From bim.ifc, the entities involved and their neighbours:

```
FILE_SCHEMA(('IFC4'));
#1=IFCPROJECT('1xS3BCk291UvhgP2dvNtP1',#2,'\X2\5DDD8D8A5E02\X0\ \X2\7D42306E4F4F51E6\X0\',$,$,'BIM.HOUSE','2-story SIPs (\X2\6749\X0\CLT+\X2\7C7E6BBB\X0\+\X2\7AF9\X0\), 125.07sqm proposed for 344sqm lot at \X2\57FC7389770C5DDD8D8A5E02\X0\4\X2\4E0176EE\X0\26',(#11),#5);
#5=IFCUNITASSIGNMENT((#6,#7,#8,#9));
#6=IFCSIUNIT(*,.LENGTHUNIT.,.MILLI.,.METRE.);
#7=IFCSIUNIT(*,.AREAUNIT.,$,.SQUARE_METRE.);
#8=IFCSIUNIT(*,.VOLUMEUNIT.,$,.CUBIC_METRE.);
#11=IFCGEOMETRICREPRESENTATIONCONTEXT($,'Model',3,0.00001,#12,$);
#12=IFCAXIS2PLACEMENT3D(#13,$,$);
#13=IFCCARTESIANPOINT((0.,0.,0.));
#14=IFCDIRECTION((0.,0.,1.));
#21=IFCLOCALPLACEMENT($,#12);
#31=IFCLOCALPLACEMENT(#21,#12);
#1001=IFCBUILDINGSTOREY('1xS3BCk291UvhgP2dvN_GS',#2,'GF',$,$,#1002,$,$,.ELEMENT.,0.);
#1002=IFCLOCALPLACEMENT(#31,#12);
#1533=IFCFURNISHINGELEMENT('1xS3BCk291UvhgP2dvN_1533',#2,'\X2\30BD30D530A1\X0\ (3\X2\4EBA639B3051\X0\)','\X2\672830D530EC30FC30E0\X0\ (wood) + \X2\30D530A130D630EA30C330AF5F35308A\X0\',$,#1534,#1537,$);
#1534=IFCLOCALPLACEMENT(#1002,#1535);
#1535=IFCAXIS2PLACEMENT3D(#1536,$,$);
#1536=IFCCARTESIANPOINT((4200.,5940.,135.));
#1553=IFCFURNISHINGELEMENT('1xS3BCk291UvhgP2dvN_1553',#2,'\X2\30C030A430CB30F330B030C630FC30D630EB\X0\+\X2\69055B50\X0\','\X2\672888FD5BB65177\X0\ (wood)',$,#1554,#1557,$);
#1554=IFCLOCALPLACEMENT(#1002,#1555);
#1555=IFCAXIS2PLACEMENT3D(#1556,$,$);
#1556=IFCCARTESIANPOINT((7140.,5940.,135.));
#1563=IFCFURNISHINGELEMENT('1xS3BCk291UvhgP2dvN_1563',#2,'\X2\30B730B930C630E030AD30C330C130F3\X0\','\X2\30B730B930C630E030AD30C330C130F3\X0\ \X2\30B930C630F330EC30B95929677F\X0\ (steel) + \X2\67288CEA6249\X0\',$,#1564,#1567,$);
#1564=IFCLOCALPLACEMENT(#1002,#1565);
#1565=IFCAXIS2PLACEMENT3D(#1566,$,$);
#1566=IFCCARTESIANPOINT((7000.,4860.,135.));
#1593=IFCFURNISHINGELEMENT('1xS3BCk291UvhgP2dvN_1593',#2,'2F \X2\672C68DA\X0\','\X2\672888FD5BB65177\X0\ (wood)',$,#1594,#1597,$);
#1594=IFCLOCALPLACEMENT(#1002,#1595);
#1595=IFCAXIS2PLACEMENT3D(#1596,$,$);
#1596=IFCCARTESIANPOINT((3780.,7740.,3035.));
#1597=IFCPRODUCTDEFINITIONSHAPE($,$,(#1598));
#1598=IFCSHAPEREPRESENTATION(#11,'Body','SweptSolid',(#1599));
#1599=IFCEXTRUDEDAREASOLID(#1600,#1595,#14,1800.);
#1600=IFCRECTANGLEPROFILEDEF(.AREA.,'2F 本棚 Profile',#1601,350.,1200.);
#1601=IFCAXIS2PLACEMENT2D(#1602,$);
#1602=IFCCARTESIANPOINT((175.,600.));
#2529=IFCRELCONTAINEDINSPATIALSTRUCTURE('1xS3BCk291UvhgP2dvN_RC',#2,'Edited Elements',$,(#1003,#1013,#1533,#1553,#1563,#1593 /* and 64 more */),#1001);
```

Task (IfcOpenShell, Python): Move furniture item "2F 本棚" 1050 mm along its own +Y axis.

```python
import ifcopenshell
import ifcopenshell.api.geometry
import ifcopenshell.util.placement
import ifcopenshell.util.unit

model = ifcopenshell.open("bim.ifc")
unit_scale = ifcopenshell.util.unit.calculate_unit_scale(model)

item = model.by_id(1593)
matrix = ifcopenshell.util.placement.get_local_placement(item.ObjectPlacement)
matrix[:3, 3] += matrix[:3, 1] * 1.05 / unit_scale
ifcopenshell.api.geometry.edit_object_placement(model, product=item, matrix=matrix, is_si=False)

print(ifcopenshell.util.placement.get_local_placement(item.ObjectPlacement).round(3) + 0.0)

model.write("bim-out.ifc")
```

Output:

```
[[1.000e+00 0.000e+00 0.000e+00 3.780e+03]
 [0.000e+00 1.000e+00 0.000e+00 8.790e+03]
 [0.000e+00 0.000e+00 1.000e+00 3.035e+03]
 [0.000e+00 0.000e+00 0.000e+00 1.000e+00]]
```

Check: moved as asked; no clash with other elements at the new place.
